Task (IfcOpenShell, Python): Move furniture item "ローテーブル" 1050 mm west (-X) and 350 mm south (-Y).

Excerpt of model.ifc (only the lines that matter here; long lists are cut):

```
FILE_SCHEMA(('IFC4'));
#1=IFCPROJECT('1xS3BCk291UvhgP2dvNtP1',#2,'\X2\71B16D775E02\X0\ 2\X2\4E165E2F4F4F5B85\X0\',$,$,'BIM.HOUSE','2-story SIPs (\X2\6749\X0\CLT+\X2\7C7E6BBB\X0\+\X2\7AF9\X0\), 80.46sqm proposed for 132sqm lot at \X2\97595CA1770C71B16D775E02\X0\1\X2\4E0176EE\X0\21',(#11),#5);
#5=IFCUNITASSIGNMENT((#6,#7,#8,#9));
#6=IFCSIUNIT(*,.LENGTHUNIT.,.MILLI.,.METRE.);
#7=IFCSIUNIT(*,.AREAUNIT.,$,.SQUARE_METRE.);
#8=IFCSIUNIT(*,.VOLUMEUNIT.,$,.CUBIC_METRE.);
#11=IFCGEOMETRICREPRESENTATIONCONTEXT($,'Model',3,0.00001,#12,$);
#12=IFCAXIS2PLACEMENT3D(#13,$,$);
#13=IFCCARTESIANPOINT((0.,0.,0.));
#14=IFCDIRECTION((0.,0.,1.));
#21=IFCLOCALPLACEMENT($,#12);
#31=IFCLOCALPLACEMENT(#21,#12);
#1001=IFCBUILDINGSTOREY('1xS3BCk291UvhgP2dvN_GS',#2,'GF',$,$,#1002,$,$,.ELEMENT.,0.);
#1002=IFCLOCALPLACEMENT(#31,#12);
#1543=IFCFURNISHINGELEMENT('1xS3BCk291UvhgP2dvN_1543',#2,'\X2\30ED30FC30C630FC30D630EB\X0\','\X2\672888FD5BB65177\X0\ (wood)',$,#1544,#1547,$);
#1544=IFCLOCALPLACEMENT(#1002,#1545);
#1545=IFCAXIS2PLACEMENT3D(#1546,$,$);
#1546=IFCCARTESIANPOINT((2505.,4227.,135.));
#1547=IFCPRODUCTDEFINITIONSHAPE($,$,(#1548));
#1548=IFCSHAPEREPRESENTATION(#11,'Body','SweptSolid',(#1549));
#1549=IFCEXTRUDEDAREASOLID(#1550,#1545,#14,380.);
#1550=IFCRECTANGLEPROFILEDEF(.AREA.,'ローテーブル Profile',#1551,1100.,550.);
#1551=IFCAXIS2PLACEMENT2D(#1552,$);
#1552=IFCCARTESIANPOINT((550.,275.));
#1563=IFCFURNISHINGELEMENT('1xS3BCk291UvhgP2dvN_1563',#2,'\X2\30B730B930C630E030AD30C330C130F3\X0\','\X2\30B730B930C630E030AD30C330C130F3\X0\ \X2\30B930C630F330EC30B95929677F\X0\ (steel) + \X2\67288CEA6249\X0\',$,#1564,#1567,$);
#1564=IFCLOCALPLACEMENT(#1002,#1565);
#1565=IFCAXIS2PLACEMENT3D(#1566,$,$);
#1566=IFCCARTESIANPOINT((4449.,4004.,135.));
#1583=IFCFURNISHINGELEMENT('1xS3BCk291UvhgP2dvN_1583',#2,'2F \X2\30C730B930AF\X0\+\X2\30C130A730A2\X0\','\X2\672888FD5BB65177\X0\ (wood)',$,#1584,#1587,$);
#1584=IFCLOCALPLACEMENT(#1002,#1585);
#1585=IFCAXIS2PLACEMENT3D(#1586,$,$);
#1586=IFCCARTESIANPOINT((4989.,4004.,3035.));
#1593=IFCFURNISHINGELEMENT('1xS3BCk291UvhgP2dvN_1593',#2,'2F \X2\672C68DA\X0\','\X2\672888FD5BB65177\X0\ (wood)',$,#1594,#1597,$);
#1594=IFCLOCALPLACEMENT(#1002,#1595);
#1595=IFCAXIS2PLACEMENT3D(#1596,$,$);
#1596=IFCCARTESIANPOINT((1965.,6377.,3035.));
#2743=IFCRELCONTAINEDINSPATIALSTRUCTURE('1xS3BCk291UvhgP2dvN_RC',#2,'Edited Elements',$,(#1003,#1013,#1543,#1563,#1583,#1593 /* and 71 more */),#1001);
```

```python
import ifcopenshell
import ifcopenshell.api.geometry
import ifcopenshell.util.placement
import ifcopenshell.util.unit

model = ifcopenshell.open("model.ifc")
unit_scale = ifcopenshell.util.unit.calculate_unit_scale(model)

item = model.by_id(1543)
matrix = ifcopenshell.util.placement.get_local_placement(item.ObjectPlacement)
matrix[0, 3] -= 1.05 / unit_scale
matrix[1, 3] -= 0.35 / unit_scale
ifcopenshell.api.geometry.edit_object_placement(model, product=item, matrix=matrix, is_si=False)

print(ifcopenshell.util.placement.get_local_placement(item.ObjectPlacement).round(3) + 0.0)

model.write("model_v2.ifc")
```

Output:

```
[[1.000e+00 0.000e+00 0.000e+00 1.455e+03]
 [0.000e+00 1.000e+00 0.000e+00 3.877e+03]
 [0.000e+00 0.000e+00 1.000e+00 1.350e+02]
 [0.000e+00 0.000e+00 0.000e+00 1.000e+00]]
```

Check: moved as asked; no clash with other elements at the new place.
